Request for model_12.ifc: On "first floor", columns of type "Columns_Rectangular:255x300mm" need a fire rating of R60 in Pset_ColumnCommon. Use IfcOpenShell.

First a look at what the model holds.

```python
import ifcopenshell
import ifcopenshell.util.element

model = ifcopenshell.open("model_12.ifc")
print(model.schema)
storey = next(s for s in model.by_type("IfcBuildingStorey") if s.Name == "first floor")
columns = [e for e in ifcopenshell.util.element.get_decomposition(storey) if e.is_a("IfcColumn")]
seen = {}
for e in columns:
    element_type = ifcopenshell.util.element.get_type(e)
    key = (element_type.Name if element_type != e and element_type else None, ifcopenshell.util.element.get_pset(e, "Pset_ColumnCommon", "FireRating"))
    seen[key] = seen.get(key, 0) + 1
for (name, value), count in sorted(seen.items(), key=str):
    print(count, "x", name, "|", value)
```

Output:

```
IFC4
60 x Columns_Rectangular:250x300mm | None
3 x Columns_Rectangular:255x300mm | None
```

```python
import ifcopenshell
import ifcopenshell.api.pset
import ifcopenshell.util.element

model = ifcopenshell.open("model_12.ifc")

storey = next(s for s in model.by_type("IfcBuildingStorey") if s.Name == "first floor")
columns = [e for e in ifcopenshell.util.element.get_decomposition(storey) if e.is_a("IfcColumn")]

count = 0
for e in columns:
    element_type = ifcopenshell.util.element.get_type(e)
    if element_type in (None, e) or element_type.Name != "Columns_Rectangular:255x300mm":
        continue
    # add_pset returns the element's existing set when there is one.
    pset = ifcopenshell.api.pset.add_pset(model, product=e, name="Pset_ColumnCommon")
    ifcopenshell.api.pset.edit_pset(model, pset=pset, properties={"FireRating": "R60"})
    count += 1

print(count, "columns updated")

model.write("model_12_edited.ifc")
```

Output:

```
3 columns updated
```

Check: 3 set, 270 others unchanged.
